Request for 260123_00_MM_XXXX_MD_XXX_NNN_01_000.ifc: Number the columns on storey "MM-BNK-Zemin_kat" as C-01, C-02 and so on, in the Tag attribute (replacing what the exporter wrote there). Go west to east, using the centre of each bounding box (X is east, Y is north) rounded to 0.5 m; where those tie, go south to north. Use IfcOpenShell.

First a look at what the model holds.

```python
import ifcopenshell
import ifcopenshell.util.element
import ifcopenshell.util.placement

model = ifcopenshell.open("260123_00_MM_XXXX_MD_XXX_NNN_01_000.ifc")
print(model.schema)
storey = next(s for s in model.by_type("IfcBuildingStorey") if s.Name == "MM-BNK-Zemin_kat")
columns = [e for e in ifcopenshell.util.element.get_decomposition(storey) if e.is_a("IfcColumn")]
for e in sorted(columns, key=lambda e: e.id()):
    origin = ifcopenshell.util.placement.get_local_placement(e.ObjectPlacement)[:3, 3]
    print(e.id(), e.Tag, e.Name, origin.round(2) + 0.0, sep=" | ")
```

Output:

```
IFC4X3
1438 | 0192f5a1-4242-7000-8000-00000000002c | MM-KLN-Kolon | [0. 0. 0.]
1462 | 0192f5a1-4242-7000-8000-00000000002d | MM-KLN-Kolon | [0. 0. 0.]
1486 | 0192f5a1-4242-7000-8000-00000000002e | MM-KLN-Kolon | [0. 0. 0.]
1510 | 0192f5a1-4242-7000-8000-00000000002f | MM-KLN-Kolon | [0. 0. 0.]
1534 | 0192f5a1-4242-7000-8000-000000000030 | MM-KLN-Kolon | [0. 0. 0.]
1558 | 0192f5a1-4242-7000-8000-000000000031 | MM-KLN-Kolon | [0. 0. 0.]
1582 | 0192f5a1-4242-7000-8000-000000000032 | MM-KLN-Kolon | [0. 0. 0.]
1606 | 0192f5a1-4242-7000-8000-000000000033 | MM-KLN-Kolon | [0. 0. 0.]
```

```python
import ifcopenshell
import ifcopenshell.geom
import ifcopenshell.util.element
import ifcopenshell.util.shape

model = ifcopenshell.open("260123_00_MM_XXXX_MD_XXX_NNN_01_000.ifc")
settings = ifcopenshell.geom.settings()
settings.set("use-world-coords", True)


def centre(element):
    shape = ifcopenshell.geom.create_shape(settings, element)
    return ifcopenshell.util.shape.get_bbox_centroid(shape.geometry)


storey = next(s for s in model.by_type("IfcBuildingStorey") if s.Name == "MM-BNK-Zemin_kat")
columns = [e for e in ifcopenshell.util.element.get_decomposition(storey) if e.is_a("IfcColumn")]

# Insertion points can sit at a corner or the storey origin, so sort by the geometry (in metres).
centres = {e: centre(e) for e in columns}
columns.sort(key=lambda e: (round(centres[e][0] / 0.5), centres[e][1]))

for i, e in enumerate(columns, start=1):
    number = f"C-{i:02d}"
    e.Tag = number
    print(e.id(), number)

model.write("260123_00_MM_XXXX_MD_XXX_NNN_01_000_rev.ifc")
```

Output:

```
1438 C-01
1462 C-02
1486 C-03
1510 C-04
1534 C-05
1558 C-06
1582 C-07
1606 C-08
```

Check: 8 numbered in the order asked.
